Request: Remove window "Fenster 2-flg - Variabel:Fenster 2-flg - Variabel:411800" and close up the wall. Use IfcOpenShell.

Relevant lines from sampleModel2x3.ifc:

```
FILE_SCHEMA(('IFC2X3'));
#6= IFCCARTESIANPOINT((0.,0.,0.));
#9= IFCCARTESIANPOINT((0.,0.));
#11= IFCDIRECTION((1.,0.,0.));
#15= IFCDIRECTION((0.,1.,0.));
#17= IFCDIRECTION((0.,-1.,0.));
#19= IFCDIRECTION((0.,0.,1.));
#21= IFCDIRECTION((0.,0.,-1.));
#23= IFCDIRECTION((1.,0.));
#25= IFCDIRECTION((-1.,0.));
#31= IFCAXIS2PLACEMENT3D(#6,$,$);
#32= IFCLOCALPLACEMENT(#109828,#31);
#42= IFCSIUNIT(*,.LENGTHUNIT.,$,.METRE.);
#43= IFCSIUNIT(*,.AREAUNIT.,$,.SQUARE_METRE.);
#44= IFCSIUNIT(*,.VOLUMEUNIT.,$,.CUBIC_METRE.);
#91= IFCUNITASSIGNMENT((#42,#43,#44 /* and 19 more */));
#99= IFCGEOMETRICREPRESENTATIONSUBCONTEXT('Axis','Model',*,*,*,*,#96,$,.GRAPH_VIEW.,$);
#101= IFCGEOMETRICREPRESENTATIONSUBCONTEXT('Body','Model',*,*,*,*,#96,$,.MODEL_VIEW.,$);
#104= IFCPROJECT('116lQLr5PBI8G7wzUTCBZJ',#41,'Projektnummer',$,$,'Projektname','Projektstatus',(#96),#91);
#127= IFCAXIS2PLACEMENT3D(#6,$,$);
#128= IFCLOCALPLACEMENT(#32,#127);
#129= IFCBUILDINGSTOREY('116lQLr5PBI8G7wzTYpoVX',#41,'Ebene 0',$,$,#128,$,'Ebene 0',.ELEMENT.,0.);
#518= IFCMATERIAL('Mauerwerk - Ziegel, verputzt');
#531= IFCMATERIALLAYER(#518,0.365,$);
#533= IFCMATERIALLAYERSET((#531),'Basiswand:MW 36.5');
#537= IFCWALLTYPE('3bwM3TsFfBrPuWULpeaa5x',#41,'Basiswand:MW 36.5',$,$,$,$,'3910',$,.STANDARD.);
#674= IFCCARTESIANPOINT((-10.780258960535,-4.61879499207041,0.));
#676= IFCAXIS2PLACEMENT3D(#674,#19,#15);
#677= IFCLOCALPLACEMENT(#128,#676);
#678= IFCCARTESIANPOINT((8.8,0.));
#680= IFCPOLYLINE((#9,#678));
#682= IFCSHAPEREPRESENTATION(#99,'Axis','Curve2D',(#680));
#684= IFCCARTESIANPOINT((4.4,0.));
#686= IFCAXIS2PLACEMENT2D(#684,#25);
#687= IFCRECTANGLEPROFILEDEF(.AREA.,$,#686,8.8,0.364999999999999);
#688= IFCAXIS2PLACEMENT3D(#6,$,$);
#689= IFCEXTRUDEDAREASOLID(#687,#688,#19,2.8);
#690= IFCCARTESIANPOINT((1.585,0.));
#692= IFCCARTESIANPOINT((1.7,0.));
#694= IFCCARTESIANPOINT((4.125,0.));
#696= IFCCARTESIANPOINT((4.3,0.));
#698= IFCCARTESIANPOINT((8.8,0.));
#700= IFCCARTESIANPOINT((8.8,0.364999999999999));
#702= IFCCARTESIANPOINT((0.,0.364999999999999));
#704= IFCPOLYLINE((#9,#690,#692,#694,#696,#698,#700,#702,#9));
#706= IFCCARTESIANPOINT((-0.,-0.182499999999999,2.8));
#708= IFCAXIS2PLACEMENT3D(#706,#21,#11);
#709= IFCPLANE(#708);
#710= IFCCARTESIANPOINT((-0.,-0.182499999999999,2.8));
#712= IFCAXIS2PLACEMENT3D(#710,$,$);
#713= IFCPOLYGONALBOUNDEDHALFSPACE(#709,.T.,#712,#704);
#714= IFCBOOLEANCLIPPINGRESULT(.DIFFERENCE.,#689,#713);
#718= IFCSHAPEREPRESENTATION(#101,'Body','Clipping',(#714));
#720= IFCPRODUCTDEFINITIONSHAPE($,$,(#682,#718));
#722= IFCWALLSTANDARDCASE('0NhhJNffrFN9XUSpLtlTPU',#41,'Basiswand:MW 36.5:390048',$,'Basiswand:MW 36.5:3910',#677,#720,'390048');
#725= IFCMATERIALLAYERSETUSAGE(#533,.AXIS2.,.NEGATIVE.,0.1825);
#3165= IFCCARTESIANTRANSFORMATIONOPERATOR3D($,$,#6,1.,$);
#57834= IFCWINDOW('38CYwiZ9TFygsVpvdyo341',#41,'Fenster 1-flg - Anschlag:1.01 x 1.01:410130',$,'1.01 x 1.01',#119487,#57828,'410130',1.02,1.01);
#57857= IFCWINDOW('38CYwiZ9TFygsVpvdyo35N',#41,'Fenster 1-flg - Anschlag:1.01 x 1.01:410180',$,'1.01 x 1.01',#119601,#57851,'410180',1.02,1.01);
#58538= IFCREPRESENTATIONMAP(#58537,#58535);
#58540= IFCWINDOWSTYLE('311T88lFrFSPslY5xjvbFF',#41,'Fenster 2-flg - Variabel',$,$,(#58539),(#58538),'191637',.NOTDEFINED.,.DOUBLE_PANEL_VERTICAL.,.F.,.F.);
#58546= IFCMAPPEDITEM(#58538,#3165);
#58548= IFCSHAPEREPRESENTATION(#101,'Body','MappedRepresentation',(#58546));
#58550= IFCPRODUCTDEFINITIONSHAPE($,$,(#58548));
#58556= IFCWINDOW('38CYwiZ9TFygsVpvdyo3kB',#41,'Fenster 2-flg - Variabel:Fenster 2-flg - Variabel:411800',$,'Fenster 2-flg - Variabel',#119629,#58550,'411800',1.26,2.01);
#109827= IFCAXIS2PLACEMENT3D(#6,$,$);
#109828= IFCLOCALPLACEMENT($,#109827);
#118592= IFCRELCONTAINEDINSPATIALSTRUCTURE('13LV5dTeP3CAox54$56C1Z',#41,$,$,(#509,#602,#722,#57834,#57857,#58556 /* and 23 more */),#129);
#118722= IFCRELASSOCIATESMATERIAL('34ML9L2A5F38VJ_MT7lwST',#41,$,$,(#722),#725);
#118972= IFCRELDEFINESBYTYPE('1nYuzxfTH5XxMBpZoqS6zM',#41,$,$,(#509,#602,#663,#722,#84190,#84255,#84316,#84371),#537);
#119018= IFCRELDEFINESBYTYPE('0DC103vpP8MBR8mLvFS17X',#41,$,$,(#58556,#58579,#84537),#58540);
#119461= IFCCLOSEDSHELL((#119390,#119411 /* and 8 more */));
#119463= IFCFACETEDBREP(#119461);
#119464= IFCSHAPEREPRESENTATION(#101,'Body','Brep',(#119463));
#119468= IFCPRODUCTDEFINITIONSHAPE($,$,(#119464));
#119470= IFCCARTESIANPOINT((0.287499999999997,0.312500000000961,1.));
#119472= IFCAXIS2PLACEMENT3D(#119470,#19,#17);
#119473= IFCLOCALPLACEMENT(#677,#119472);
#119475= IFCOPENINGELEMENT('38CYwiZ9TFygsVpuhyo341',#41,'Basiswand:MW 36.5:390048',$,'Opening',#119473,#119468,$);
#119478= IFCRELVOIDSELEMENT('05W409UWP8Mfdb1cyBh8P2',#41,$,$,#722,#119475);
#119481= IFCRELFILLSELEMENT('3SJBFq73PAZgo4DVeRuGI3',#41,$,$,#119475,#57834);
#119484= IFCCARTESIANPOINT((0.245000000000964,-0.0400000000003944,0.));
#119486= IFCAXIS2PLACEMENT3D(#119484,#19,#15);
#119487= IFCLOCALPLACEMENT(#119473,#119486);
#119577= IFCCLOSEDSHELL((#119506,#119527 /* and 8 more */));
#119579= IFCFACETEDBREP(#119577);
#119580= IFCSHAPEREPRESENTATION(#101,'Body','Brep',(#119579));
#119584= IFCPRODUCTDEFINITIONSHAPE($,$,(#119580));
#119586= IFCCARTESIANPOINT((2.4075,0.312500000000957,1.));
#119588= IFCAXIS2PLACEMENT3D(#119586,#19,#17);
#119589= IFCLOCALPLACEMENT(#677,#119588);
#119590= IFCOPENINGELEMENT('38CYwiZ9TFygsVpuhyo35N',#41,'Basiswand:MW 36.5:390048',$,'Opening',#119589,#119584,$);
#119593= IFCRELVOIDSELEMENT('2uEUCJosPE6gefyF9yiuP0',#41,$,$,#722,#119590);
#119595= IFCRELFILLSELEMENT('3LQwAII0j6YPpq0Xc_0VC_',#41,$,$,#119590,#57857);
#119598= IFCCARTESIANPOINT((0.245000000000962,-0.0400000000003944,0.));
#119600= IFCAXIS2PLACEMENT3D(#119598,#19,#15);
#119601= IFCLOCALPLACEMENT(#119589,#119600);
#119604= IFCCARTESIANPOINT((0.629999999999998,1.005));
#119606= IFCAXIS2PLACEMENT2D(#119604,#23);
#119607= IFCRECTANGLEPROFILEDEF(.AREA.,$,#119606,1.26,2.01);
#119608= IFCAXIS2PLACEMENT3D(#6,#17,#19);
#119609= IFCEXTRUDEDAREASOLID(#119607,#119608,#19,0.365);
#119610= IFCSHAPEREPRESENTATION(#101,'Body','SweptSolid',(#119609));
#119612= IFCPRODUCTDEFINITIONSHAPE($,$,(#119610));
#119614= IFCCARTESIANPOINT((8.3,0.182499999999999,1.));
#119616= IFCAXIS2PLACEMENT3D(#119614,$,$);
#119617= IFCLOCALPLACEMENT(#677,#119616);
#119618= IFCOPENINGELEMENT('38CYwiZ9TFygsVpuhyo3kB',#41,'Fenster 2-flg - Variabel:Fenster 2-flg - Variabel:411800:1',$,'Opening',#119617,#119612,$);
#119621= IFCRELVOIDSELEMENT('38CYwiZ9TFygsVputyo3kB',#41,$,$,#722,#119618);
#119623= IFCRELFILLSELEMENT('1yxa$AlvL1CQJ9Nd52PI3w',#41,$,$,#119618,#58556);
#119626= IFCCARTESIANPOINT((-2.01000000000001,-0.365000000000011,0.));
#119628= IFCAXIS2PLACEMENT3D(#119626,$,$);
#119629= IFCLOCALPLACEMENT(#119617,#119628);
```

```python
import ifcopenshell
import ifcopenshell.api.feature
import ifcopenshell.api.root
import ifcopenshell.geom
import ifcopenshell.util.shape

model = ifcopenshell.open("sampleModel2x3.ifc")
settings = ifcopenshell.geom.settings()


def volume(element):
    """Net volume in cubic metres, openings subtracted."""
    shape = ifcopenshell.geom.create_shape(settings, element)
    return ifcopenshell.util.shape.get_volume(shape.geometry)


window = model.by_id(58556)
opening = window.FillsVoids[0].RelatingOpeningElement
wall = opening.VoidsElements[0].RelatingBuildingElement
before = volume(wall)

ifcopenshell.api.root.remove_product(model, product=window)
ifcopenshell.api.feature.remove_feature(model, feature=opening)

after = volume(wall)

print(f"wall volume {before:.3f} -> {after:.3f} m3")

model.write("sampleModel2x3_rev.ifc")
```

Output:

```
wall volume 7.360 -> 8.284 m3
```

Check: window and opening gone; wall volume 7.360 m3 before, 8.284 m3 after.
